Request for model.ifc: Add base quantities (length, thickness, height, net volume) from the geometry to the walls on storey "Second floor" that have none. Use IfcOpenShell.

First a look at what the model holds.

```python
import ifcopenshell
import ifcopenshell.util.element
import ifcopenshell.util.unit

model = ifcopenshell.open("model.ifc")
print(model.schema)
for unit_type in ("LENGTHUNIT", "AREAUNIT", "VOLUMEUNIT"):
    print(unit_type, ifcopenshell.util.unit.calculate_unit_scale(model, unit_type))
storey = next(s for s in model.by_type("IfcBuildingStorey") if s.Name == "Second floor")
walls = [e for e in ifcopenshell.util.element.get_decomposition(storey) if e.is_a("IfcWall")]
for e in sorted(walls, key=lambda e: e.id()):
    print(e.id(), e.is_a(), e.Name, list(ifcopenshell.util.element.get_psets(e, qtos_only=True)), sep=" | ")
```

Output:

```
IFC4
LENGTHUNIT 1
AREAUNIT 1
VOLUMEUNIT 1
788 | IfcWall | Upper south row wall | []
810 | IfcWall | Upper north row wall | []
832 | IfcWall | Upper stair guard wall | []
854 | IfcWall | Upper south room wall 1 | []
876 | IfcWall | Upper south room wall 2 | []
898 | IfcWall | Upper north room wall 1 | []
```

```python
import ifcopenshell
import ifcopenshell.api.pset
import ifcopenshell.geom
import ifcopenshell.util.element
import ifcopenshell.util.shape
import ifcopenshell.util.unit

model = ifcopenshell.open("model.ifc")
unit_scale = ifcopenshell.util.unit.calculate_unit_scale(model)
volume_scale = ifcopenshell.util.unit.calculate_unit_scale(model, "VOLUMEUNIT")
settings = ifcopenshell.geom.settings()

storey = next(s for s in model.by_type("IfcBuildingStorey") if s.Name == "Second floor")
walls = [e for e in ifcopenshell.util.element.get_decomposition(storey) if e.is_a("IfcWall")]

for e in sorted(walls, key=lambda e: e.id()):
    if ifcopenshell.util.element.get_psets(e, qtos_only=True, should_inherit=False):
        continue
    # Geometry comes back in metres, in the element's own axes.
    shape = ifcopenshell.geom.create_shape(settings, e)
    values = {
        "Length": ifcopenshell.util.shape.get_x(shape.geometry) / unit_scale,
        "Width": ifcopenshell.util.shape.get_y(shape.geometry) / unit_scale,
        "Height": ifcopenshell.util.shape.get_z(shape.geometry) / unit_scale,
        "NetVolume": ifcopenshell.util.shape.get_volume(shape.geometry) / volume_scale,
    }
    qto = ifcopenshell.api.pset.add_qto(model, product=e, name="Qto_WallBaseQuantities")
    ifcopenshell.api.pset.edit_qto(model, qto=qto, properties=values)
    print(e.id(), {k: round(v, 3) for k, v in values.items()})

model.write("model_updated.ifc")
```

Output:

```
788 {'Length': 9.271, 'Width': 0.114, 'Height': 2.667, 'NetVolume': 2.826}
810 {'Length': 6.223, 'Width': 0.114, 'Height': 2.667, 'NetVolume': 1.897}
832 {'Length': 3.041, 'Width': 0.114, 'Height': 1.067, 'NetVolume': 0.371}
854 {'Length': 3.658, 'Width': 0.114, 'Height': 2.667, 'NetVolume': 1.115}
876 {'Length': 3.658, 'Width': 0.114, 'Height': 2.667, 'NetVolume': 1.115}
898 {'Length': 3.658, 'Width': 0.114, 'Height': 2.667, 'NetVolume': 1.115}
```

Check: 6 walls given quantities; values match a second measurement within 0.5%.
